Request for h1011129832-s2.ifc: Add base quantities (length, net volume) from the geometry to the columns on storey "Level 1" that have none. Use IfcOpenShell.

First a look at what the model holds.

```python
import ifcopenshell
import ifcopenshell.util.element
import ifcopenshell.util.unit

model = ifcopenshell.open("h1011129832-s2.ifc")
print(model.schema)
for unit_type in ("LENGTHUNIT", "AREAUNIT", "VOLUMEUNIT"):
    print(unit_type, ifcopenshell.util.unit.calculate_unit_scale(model, unit_type))
storey = next(s for s in model.by_type("IfcBuildingStorey") if s.Name == "Level 1")
columns = [e for e in ifcopenshell.util.element.get_decomposition(storey) if e.is_a("IfcColumn")]
for e in sorted(columns, key=lambda e: e.id()):
    print(e.id(), e.is_a(), e.Name, list(ifcopenshell.util.element.get_psets(e, qtos_only=True)), sep=" | ")
```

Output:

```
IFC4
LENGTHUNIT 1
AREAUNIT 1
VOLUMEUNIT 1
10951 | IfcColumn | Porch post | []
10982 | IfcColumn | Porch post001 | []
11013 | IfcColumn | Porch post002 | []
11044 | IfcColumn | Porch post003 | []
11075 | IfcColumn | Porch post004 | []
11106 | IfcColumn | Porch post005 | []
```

```python
import ifcopenshell
import ifcopenshell.api.pset
import ifcopenshell.geom
import ifcopenshell.util.element
import ifcopenshell.util.shape
import ifcopenshell.util.unit

model = ifcopenshell.open("h1011129832-s2.ifc")
unit_scale = ifcopenshell.util.unit.calculate_unit_scale(model)
volume_scale = ifcopenshell.util.unit.calculate_unit_scale(model, "VOLUMEUNIT")
settings = ifcopenshell.geom.settings()

storey = next(s for s in model.by_type("IfcBuildingStorey") if s.Name == "Level 1")
columns = [e for e in ifcopenshell.util.element.get_decomposition(storey) if e.is_a("IfcColumn")]

for e in sorted(columns, key=lambda e: e.id()):
    if ifcopenshell.util.element.get_psets(e, qtos_only=True, should_inherit=False):
        continue
    # Geometry comes back in metres, in the element's own axes.
    shape = ifcopenshell.geom.create_shape(settings, e)
    values = {
        "Length": ifcopenshell.util.shape.get_z(shape.geometry) / unit_scale,
        "NetVolume": ifcopenshell.util.shape.get_volume(shape.geometry) / volume_scale,
    }
    qto = ifcopenshell.api.pset.add_qto(model, product=e, name="Qto_ColumnBaseQuantities")
    ifcopenshell.api.pset.edit_qto(model, qto=qto, properties=values)
    print(e.id(), {k: round(v, 3) for k, v in values.items()})

model.write("h1011129832-s2_updated.ifc")
```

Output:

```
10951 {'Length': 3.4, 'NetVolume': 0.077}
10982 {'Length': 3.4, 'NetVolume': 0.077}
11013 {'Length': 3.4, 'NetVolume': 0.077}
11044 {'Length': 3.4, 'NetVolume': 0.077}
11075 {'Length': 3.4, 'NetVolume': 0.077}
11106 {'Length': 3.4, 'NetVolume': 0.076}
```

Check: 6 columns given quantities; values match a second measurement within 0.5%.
